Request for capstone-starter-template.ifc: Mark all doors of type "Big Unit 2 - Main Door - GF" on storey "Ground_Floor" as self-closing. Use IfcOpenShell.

First a look at what the model holds.

```python
import ifcopenshell
import ifcopenshell.util.element

model = ifcopenshell.open("capstone-starter-template.ifc")
print(model.schema)
storey = next(s for s in model.by_type("IfcBuildingStorey") if s.Name == "Ground_Floor")
doors = [e for e in ifcopenshell.util.element.get_decomposition(storey) if e.is_a("IfcDoor")]
seen = {}
for e in doors:
    element_type = ifcopenshell.util.element.get_type(e)
    key = (element_type.Name if element_type != e and element_type else None, ifcopenshell.util.element.get_pset(e, "Pset_DoorCommon", "SelfClosing"))
    seen[key] = seen.get(key, 0) + 1
for (name, value), count in sorted(seen.items(), key=str):
    print(count, "x", name, "|", value)
```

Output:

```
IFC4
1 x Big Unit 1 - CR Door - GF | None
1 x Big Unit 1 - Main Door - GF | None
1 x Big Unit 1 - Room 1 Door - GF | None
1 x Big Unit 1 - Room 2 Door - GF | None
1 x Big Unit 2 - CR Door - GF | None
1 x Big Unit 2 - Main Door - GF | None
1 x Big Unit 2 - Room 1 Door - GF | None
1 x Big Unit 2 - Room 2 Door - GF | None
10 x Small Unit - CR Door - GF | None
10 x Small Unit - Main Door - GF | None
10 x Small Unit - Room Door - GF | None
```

```python
import ifcopenshell
import ifcopenshell.api.pset
import ifcopenshell.util.element

model = ifcopenshell.open("capstone-starter-template.ifc")

storey = next(s for s in model.by_type("IfcBuildingStorey") if s.Name == "Ground_Floor")
doors = [e for e in ifcopenshell.util.element.get_decomposition(storey) if e.is_a("IfcDoor")]

count = 0
for e in doors:
    element_type = ifcopenshell.util.element.get_type(e)
    if element_type in (None, e) or element_type.Name != "Big Unit 2 - Main Door - GF":
        continue
    # add_pset returns the element's existing set when there is one.
    pset = ifcopenshell.api.pset.add_pset(model, product=e, name="Pset_DoorCommon")
    ifcopenshell.api.pset.edit_pset(model, pset=pset, properties={"SelfClosing": True})
    count += 1

print(count, "doors updated")

model.write("capstone-starter-template_rev.ifc")
```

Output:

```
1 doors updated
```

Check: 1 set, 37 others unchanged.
